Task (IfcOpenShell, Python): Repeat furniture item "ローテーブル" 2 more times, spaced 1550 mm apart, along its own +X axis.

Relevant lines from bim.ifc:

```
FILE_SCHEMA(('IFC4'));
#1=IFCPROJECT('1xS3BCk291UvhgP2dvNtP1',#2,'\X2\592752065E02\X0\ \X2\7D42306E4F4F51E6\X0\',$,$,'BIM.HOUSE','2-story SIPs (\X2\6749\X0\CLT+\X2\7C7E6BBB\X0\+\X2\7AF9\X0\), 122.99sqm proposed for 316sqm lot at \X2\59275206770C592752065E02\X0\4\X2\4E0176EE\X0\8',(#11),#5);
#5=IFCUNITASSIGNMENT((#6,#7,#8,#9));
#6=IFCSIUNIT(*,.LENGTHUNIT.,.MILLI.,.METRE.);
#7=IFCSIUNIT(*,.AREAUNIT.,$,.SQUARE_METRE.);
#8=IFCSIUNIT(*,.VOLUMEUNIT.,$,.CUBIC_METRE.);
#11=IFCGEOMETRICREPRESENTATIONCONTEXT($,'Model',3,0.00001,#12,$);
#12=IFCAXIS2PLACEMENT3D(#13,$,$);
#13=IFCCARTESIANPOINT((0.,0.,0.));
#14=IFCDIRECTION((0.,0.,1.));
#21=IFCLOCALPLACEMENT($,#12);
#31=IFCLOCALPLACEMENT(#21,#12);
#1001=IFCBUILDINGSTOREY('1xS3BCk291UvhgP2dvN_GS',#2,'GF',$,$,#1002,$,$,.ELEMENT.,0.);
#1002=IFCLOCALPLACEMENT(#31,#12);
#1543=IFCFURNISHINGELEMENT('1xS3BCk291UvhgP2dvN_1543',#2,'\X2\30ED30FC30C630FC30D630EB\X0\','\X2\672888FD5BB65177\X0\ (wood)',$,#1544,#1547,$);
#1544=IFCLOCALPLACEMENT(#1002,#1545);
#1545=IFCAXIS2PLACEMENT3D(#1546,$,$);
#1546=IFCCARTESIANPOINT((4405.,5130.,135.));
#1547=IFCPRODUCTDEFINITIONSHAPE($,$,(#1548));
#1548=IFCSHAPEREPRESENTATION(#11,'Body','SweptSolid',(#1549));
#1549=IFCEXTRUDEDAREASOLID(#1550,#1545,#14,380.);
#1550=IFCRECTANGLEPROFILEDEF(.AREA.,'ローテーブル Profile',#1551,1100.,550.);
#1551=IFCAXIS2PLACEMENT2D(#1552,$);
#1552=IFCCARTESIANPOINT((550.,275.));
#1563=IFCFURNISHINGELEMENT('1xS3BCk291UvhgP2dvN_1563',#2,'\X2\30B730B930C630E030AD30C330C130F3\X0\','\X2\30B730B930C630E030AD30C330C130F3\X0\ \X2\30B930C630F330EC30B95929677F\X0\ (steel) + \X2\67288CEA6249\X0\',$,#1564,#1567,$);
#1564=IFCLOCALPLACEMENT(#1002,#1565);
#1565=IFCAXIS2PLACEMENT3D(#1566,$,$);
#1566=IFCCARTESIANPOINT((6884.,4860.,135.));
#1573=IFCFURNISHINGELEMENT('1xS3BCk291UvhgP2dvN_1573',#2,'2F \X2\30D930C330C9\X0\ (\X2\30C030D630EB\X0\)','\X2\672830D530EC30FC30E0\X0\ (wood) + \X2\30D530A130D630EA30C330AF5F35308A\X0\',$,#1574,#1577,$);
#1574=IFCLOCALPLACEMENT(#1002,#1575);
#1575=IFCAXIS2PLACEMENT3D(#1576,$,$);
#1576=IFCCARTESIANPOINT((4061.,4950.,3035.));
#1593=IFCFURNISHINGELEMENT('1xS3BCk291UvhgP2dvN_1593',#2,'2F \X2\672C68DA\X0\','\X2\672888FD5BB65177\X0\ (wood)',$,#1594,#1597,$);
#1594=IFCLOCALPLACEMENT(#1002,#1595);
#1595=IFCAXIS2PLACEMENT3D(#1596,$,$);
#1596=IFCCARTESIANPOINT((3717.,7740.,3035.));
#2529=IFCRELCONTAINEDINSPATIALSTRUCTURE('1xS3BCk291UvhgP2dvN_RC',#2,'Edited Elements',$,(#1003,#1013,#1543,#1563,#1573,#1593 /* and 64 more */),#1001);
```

```python
import ifcopenshell
import ifcopenshell.api.geometry
import ifcopenshell.api.root
import ifcopenshell.util.element
import ifcopenshell.util.placement

model = ifcopenshell.open("bim.ifc")


def reuse_history(source, copy):
    """copy_class also copies each property set's owner history, people and application; keep the originals."""
    for rel in copy.IsDefinedBy:
        if rel.is_a("IfcRelDefinesByProperties") and (history := rel.RelatingPropertyDefinition.OwnerHistory):
            rel.RelatingPropertyDefinition.OwnerHistory = source.OwnerHistory
            ifcopenshell.util.element.remove_deep2(model, history)


source = model.by_id(1543)
base = ifcopenshell.util.placement.get_local_placement(source.ObjectPlacement)
step = base[:3, 0] * 1550.0

for i in range(1, 3):
    copy = ifcopenshell.api.root.copy_class(model, product=source)
    copy.Representation = ifcopenshell.util.element.copy_deep(
        model, source.Representation, exclude=["IfcGeometricRepresentationContext", "IfcRepresentationMap"]
    )
    reuse_history(source, copy)
    matrix = base.copy()
    matrix[:3, 3] += i * step
    print("added at", matrix[:3, 3].round(3) + 0.0)
    ifcopenshell.api.geometry.edit_object_placement(model, product=copy, matrix=matrix, is_si=False)

model.write("bim_v2.ifc")
```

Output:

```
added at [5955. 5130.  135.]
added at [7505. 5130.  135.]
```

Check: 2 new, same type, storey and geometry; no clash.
